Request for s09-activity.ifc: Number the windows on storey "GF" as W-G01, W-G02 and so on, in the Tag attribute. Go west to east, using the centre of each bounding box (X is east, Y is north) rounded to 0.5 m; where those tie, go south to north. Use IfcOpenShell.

First a look at what the model holds.

```python
import ifcopenshell
import ifcopenshell.util.element
import ifcopenshell.util.placement

model = ifcopenshell.open("s09-activity.ifc")
print(model.schema)
storey = next(s for s in model.by_type("IfcBuildingStorey") if s.Name == "GF")
windows = [e for e in ifcopenshell.util.element.get_decomposition(storey) if e.is_a("IfcWindow")]
for e in sorted(windows, key=lambda e: e.id()):
    origin = ifcopenshell.util.placement.get_local_placement(e.ObjectPlacement)[:3, 3]
    print(e.id(), e.Tag, e.Name, origin.round(2) + 0.0, sep=" | ")
```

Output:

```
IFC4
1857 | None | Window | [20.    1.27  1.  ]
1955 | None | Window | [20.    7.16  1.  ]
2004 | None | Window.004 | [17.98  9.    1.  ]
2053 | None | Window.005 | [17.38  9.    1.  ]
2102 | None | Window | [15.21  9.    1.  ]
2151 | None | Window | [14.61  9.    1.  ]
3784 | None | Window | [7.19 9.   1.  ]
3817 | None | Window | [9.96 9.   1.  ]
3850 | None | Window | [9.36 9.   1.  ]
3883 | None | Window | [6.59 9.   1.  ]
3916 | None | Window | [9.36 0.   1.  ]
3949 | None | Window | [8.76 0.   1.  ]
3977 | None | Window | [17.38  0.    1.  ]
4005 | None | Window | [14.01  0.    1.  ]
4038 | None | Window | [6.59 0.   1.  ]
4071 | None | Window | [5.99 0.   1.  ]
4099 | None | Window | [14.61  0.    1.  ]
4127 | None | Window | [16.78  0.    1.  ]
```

```python
import ifcopenshell
import ifcopenshell.geom
import ifcopenshell.util.element
import ifcopenshell.util.shape

model = ifcopenshell.open("s09-activity.ifc")
settings = ifcopenshell.geom.settings()
settings.set("use-world-coords", True)


def centre(element):
    shape = ifcopenshell.geom.create_shape(settings, element)
    return ifcopenshell.util.shape.get_bbox_centroid(shape.geometry)


storey = next(s for s in model.by_type("IfcBuildingStorey") if s.Name == "GF")
windows = [e for e in ifcopenshell.util.element.get_decomposition(storey) if e.is_a("IfcWindow")]

# Insertion points can sit at a corner or the storey origin, so sort by the geometry (in metres).
centres = {e: centre(e) for e in windows}
windows.sort(key=lambda e: (round(centres[e][0] / 0.5), centres[e][1]))

for i, e in enumerate(windows, start=1):
    number = f"W-G{i:02d}"
    e.Tag = number
    print(e.id(), number)

model.write("s09-activity_rev.ifc")
```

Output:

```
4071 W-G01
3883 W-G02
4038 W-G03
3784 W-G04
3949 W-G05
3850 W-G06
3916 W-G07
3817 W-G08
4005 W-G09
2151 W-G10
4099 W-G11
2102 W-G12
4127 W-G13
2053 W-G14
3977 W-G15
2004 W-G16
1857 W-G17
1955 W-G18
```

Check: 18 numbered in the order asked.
